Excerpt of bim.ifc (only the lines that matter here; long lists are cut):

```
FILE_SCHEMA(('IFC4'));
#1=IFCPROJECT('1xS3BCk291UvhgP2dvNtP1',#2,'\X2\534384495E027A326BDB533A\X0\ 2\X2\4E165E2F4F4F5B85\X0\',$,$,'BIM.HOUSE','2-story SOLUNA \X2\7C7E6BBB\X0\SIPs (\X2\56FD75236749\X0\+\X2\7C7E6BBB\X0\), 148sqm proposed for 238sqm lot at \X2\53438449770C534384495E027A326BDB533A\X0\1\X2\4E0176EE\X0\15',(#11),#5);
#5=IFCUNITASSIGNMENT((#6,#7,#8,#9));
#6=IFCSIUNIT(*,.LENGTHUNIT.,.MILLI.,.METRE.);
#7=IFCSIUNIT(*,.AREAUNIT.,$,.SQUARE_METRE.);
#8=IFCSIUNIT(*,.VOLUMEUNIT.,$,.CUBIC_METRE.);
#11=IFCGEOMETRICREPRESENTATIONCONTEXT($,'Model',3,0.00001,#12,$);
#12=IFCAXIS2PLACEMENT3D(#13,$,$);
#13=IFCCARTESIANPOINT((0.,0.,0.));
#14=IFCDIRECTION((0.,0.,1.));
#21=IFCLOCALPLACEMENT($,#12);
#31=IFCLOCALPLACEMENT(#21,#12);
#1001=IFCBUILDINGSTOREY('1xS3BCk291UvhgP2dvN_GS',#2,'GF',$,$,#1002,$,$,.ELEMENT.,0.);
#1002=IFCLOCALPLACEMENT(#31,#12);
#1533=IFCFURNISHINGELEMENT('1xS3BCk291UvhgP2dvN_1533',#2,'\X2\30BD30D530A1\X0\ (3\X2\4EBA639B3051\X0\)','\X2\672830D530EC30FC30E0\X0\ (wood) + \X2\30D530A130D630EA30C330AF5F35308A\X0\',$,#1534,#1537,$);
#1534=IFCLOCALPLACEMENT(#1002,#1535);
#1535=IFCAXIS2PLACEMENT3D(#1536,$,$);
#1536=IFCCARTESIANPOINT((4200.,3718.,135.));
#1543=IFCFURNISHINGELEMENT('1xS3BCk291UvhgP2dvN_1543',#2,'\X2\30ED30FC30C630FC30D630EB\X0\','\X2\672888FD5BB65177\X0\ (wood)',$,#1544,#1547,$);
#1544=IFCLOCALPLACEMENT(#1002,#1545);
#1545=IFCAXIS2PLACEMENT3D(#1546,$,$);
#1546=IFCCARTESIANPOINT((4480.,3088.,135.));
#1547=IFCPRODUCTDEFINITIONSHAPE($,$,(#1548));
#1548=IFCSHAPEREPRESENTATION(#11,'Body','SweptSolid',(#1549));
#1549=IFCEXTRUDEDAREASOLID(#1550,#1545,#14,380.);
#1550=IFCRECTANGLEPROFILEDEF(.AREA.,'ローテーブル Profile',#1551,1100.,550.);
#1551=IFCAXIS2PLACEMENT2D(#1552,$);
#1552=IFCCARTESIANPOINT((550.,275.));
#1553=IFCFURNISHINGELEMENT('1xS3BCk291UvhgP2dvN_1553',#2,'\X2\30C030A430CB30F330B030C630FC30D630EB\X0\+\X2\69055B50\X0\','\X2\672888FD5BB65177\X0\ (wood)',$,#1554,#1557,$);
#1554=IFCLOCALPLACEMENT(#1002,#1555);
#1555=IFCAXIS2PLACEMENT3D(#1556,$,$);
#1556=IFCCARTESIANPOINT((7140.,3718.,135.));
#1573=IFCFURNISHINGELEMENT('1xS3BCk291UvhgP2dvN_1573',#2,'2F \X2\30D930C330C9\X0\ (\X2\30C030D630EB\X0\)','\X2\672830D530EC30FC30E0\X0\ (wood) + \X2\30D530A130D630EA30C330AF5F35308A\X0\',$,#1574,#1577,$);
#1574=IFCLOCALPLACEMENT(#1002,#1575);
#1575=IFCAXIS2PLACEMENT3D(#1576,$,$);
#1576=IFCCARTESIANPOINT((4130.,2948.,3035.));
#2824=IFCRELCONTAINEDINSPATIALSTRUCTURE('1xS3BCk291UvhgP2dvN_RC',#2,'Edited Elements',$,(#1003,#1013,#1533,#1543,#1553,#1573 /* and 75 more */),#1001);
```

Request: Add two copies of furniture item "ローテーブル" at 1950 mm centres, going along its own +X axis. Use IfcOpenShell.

```python
import ifcopenshell
import ifcopenshell.api.geometry
import ifcopenshell.api.root
import ifcopenshell.util.element
import ifcopenshell.util.placement

model = ifcopenshell.open("bim.ifc")


def reuse_history(source, copy):
    """copy_class also copies each property set's owner history, people and application; keep the originals."""
    for rel in copy.IsDefinedBy:
        if rel.is_a("IfcRelDefinesByProperties") and (history := rel.RelatingPropertyDefinition.OwnerHistory):
            rel.RelatingPropertyDefinition.OwnerHistory = source.OwnerHistory
            ifcopenshell.util.element.remove_deep2(model, history)


source = model.by_guid("1xS3BCk291UvhgP2dvN_1543")
base = ifcopenshell.util.placement.get_local_placement(source.ObjectPlacement)
step = base[:3, 0] * 1950.0

for i in range(1, 3):
    copy = ifcopenshell.api.root.copy_class(model, product=source)
    copy.Representation = ifcopenshell.util.element.copy_deep(
        model, source.Representation, exclude=["IfcGeometricRepresentationContext", "IfcRepresentationMap"]
    )
    reuse_history(source, copy)
    matrix = base.copy()
    matrix[:3, 3] += i * step
    print("added at", matrix[:3, 3].round(3) + 0.0)
    ifcopenshell.api.geometry.edit_object_placement(model, product=copy, matrix=matrix, is_si=False)

model.write("bim_v2.ifc")
```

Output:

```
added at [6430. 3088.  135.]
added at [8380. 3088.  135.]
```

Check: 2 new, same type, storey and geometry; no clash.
